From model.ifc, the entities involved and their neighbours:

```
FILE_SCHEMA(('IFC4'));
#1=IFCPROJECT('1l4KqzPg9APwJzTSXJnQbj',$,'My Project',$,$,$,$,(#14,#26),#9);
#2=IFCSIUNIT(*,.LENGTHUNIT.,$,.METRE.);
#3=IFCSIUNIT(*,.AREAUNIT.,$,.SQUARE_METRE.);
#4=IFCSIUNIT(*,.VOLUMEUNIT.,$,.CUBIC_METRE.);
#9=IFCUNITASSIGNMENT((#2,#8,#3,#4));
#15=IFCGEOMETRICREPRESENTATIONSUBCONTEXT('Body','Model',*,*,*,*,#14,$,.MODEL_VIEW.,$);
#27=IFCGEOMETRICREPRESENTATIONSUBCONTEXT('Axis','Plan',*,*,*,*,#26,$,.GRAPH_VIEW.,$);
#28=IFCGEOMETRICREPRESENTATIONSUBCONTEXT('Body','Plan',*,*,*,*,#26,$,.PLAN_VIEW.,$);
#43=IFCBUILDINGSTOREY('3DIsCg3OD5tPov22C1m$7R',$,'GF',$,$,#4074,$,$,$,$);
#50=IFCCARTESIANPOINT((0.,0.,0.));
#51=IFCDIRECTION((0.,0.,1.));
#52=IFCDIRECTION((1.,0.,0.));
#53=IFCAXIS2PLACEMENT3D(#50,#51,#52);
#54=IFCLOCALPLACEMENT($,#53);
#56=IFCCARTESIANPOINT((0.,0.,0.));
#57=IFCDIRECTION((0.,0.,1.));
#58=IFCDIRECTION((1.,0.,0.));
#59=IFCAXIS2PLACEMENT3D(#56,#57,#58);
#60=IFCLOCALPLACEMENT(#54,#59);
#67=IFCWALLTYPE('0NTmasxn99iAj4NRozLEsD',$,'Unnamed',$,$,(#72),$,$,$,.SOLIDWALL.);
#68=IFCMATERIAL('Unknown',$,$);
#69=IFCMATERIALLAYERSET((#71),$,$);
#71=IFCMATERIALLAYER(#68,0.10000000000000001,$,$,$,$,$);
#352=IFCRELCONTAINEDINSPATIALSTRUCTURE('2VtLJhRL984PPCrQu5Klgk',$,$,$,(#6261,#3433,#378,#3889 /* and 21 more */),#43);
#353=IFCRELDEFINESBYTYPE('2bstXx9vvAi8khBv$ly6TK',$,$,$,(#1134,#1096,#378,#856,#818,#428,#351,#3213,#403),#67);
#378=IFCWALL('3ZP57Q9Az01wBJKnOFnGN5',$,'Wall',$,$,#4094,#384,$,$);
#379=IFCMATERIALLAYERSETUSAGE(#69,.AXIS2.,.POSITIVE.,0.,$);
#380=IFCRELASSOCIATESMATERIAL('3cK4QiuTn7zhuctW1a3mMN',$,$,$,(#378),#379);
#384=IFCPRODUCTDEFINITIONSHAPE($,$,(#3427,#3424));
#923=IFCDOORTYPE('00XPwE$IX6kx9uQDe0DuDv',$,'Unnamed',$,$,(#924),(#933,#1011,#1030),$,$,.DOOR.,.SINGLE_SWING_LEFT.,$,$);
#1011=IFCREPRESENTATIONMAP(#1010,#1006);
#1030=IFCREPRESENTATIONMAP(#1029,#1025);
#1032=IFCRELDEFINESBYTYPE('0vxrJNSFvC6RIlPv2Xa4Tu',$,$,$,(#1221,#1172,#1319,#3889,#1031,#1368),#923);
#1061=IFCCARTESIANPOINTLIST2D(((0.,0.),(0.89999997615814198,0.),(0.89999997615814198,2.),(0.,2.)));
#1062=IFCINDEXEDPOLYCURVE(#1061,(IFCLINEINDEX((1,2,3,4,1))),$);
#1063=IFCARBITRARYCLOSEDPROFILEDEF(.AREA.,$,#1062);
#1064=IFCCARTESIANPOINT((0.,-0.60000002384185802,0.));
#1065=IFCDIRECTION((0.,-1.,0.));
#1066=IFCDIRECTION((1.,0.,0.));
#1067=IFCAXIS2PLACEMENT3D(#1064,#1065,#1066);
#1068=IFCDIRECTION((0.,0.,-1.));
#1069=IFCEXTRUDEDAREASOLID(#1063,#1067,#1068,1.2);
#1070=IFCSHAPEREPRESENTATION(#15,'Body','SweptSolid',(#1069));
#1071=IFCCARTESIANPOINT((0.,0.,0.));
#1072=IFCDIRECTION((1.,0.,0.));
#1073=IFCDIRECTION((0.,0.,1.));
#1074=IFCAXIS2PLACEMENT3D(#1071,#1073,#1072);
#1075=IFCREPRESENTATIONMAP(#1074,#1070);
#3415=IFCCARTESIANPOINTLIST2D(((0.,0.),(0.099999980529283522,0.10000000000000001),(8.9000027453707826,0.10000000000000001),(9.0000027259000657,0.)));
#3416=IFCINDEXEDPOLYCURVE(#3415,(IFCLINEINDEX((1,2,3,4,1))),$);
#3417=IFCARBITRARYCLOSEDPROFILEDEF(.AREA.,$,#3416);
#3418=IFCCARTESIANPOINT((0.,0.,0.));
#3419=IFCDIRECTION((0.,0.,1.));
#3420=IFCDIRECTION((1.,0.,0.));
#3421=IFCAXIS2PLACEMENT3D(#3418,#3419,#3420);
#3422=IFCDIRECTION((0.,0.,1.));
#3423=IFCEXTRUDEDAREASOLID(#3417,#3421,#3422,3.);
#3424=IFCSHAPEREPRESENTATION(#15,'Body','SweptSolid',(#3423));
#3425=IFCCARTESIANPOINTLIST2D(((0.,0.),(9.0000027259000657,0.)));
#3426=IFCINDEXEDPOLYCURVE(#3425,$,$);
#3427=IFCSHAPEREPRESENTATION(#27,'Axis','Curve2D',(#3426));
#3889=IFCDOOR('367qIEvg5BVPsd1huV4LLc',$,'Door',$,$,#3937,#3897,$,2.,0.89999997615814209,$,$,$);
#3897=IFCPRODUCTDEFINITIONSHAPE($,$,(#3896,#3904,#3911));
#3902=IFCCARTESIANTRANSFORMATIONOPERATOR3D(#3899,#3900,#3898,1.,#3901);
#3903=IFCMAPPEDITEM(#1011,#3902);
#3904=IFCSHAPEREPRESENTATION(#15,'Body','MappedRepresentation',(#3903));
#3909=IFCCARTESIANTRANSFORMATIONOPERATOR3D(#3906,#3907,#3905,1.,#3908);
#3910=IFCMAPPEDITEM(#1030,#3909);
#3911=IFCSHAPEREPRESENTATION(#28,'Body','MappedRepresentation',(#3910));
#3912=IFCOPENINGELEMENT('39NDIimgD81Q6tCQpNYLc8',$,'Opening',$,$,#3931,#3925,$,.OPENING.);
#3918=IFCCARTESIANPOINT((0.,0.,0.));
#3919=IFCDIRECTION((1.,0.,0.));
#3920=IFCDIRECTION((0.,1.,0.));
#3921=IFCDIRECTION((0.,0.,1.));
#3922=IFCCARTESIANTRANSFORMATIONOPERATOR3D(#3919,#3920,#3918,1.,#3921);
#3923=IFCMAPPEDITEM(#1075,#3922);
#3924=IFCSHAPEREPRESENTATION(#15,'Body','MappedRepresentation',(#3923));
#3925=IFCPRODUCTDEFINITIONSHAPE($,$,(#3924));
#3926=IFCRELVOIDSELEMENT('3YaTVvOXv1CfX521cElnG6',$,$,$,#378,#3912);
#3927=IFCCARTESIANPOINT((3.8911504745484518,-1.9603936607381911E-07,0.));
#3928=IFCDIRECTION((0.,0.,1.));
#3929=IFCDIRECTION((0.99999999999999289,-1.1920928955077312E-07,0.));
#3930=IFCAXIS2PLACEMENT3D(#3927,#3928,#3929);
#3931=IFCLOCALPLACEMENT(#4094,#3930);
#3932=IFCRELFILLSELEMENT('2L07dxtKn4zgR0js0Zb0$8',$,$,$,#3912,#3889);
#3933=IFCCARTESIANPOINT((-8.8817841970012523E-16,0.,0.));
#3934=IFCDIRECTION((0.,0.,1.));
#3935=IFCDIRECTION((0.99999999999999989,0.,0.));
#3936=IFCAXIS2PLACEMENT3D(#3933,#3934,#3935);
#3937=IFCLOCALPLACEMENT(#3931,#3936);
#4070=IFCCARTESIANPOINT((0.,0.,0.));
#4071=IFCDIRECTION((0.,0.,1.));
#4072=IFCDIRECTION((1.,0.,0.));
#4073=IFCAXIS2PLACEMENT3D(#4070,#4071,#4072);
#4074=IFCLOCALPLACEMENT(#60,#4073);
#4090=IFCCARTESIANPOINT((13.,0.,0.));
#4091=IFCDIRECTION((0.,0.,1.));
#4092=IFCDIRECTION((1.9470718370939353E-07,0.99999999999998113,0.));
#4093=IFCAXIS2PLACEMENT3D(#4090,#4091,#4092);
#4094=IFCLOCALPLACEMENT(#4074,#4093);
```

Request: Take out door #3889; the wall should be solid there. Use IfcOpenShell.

```python
import ifcopenshell
import ifcopenshell.api.feature
import ifcopenshell.api.root
import ifcopenshell.geom
import ifcopenshell.util.shape

model = ifcopenshell.open("model.ifc")
settings = ifcopenshell.geom.settings()


def volume(element):
    """Net volume in cubic metres, openings subtracted."""
    shape = ifcopenshell.geom.create_shape(settings, element)
    return ifcopenshell.util.shape.get_volume(shape.geometry)


door = model.by_guid("367qIEvg5BVPsd1huV4LLc")
opening = door.FillsVoids[0].RelatingOpeningElement
wall = opening.VoidsElements[0].RelatingBuildingElement
before = volume(wall)

ifcopenshell.api.root.remove_product(model, product=door)
ifcopenshell.api.feature.remove_feature(model, feature=opening)

after = volume(wall)

print(f"wall volume {before:.3f} -> {after:.3f} m3")

model.write("model_edited.ifc")
```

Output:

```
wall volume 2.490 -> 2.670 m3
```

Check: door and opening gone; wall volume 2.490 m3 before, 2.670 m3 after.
